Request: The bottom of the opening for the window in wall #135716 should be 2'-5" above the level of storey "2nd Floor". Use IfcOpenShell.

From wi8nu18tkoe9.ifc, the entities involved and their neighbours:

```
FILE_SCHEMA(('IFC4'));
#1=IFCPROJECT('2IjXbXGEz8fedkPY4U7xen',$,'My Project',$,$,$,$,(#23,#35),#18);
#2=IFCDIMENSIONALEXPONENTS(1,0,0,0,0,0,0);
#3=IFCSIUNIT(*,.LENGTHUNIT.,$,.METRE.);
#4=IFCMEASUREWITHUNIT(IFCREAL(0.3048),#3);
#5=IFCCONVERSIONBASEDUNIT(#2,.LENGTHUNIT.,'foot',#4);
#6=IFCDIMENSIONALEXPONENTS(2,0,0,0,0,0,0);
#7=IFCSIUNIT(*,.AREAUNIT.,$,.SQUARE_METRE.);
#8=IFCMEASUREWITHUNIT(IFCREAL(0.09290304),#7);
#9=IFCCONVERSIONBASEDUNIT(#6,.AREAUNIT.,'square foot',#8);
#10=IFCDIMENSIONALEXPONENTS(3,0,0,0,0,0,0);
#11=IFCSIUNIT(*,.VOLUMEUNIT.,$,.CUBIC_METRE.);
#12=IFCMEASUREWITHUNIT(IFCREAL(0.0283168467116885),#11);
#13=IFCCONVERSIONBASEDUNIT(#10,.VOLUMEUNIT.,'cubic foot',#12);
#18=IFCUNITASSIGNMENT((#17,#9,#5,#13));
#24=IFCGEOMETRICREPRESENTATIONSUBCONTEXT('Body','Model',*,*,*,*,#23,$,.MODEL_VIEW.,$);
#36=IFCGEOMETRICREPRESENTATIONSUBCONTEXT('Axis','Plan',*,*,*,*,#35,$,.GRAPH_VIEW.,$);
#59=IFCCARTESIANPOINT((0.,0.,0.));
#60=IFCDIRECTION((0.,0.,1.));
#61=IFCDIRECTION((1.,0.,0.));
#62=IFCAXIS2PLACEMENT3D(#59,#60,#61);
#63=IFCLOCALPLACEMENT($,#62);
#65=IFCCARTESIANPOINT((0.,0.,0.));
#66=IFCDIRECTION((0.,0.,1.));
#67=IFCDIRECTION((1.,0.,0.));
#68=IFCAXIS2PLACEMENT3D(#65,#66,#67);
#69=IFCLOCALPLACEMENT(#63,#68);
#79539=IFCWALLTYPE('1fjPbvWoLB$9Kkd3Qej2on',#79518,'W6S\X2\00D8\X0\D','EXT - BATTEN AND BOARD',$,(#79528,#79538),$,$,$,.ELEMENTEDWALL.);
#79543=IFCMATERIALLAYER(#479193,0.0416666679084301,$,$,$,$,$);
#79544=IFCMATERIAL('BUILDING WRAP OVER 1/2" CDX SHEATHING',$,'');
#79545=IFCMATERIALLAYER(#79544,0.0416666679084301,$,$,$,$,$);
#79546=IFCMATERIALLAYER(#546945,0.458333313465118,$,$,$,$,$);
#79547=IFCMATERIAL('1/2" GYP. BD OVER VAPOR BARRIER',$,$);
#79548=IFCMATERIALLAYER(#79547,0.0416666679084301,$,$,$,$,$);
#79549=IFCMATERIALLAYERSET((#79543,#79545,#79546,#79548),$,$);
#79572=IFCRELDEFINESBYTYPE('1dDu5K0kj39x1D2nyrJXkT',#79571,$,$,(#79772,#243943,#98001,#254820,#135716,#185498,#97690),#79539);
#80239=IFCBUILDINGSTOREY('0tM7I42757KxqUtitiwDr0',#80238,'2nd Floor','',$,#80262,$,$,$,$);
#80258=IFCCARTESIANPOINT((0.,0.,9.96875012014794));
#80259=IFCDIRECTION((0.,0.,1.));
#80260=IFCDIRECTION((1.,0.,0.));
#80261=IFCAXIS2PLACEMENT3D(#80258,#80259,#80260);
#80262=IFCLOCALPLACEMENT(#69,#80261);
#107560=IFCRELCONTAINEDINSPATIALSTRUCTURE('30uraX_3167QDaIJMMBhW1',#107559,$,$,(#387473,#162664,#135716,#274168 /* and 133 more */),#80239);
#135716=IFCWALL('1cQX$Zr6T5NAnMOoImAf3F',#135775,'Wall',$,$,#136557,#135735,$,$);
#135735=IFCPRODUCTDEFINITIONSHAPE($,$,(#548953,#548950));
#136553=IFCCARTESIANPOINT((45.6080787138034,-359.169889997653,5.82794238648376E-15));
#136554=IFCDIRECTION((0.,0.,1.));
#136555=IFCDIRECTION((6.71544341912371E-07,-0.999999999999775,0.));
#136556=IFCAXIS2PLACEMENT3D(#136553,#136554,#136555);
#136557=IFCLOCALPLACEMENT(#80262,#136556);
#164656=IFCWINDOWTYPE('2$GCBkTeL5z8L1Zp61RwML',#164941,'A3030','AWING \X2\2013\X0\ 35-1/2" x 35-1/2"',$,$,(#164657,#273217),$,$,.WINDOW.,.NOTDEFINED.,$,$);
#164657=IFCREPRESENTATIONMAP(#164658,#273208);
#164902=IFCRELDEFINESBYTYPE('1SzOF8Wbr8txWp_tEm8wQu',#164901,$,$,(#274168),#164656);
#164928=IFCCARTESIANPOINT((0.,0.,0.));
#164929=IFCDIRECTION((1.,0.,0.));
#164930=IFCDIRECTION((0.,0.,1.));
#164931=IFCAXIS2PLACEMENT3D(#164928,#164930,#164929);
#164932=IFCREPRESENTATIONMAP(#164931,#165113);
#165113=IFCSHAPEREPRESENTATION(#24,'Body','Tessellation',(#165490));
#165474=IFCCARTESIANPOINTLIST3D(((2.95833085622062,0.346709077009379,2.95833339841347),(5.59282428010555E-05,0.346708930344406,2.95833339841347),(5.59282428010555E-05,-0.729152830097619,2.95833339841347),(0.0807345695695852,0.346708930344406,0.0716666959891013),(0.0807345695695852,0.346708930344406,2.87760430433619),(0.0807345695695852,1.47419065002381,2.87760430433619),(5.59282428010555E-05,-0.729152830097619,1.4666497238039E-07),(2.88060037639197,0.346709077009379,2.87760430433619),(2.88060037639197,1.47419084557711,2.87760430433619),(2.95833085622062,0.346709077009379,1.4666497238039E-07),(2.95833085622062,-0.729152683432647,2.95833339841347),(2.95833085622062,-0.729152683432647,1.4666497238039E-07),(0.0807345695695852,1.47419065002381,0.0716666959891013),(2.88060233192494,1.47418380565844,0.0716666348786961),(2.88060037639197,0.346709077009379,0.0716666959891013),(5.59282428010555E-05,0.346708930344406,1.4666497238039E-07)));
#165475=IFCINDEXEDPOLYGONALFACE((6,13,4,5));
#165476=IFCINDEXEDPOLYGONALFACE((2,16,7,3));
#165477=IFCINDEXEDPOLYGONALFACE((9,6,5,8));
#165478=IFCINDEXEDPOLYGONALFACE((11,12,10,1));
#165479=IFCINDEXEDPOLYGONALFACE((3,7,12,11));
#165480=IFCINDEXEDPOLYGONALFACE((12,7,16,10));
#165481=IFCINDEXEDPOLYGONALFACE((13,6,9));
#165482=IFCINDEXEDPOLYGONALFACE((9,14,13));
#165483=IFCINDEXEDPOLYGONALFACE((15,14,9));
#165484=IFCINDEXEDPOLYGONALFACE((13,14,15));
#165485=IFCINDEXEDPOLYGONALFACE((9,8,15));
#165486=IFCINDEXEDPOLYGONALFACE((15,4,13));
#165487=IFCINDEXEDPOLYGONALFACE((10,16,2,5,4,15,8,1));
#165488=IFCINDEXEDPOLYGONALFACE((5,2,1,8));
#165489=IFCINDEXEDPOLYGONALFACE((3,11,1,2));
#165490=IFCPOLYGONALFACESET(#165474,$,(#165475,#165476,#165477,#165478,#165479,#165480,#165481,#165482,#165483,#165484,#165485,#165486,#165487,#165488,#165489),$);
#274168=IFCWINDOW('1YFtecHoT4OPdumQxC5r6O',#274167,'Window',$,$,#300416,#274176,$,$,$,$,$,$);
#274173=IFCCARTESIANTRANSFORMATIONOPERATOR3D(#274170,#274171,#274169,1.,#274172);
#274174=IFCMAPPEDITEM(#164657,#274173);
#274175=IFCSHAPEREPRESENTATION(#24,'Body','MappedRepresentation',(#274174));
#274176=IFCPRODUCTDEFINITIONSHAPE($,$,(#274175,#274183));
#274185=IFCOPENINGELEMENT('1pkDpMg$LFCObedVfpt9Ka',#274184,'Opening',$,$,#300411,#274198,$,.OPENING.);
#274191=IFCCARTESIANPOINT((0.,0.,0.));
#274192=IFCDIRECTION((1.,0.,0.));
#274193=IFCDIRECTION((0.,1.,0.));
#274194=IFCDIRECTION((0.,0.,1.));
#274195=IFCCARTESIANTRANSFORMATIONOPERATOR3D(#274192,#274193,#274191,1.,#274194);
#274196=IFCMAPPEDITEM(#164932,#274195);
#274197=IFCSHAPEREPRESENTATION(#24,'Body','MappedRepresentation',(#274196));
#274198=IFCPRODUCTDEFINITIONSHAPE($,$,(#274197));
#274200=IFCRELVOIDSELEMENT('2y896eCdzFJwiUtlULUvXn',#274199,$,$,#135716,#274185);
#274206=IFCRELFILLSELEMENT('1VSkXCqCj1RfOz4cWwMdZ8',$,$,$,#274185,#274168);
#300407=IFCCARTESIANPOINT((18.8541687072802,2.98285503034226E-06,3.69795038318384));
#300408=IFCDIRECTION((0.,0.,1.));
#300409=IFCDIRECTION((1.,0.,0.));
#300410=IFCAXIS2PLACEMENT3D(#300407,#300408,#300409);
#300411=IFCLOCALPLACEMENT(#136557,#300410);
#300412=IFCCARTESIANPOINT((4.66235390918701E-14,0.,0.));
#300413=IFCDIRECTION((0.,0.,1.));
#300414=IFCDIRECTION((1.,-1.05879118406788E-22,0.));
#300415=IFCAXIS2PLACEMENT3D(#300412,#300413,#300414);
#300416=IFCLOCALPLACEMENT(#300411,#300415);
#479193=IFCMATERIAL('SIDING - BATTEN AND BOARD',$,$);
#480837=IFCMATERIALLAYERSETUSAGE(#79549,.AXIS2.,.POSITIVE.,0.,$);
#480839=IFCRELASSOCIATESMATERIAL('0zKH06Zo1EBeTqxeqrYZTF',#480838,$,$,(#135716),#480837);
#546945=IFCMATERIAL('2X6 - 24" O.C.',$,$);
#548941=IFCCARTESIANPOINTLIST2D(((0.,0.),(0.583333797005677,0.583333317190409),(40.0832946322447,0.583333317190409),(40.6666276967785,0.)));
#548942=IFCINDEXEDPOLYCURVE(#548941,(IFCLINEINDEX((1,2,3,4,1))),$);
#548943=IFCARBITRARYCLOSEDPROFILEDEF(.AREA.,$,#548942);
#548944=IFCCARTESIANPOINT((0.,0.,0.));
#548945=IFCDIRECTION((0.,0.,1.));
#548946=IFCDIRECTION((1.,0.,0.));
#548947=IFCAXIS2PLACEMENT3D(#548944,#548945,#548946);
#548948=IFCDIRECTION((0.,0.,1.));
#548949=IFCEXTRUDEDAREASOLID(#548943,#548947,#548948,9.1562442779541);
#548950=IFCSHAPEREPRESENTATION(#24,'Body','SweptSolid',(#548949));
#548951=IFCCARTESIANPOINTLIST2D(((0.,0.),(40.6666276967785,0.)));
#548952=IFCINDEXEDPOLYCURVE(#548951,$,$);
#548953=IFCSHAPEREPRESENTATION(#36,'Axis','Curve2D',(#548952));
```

```python
import numpy as np
import ifcopenshell
import ifcopenshell.api.geometry
import ifcopenshell.geom
import ifcopenshell.util.element
import ifcopenshell.util.placement
import ifcopenshell.util.shape
import ifcopenshell.util.unit

model = ifcopenshell.open("wi8nu18tkoe9.ifc")
unit_scale = ifcopenshell.util.unit.calculate_unit_scale(model)

window = model.by_id(274168)
opening = window.FillsVoids[0].RelatingOpeningElement
storey = ifcopenshell.util.element.get_container(window, ifc_class="IfcBuildingStorey")
level = ifcopenshell.util.placement.get_local_placement(storey.ObjectPlacement)[2, 3]

# The opening's origin need not be at the sill, so measure its lowest point.
shape = ifcopenshell.geom.create_shape(ifcopenshell.geom.settings(), opening)
bottom = ifcopenshell.util.shape.get_shape_bottom_elevation(shape, shape.geometry) / unit_scale
dz = level + 29 * 0.0254 / unit_scale - bottom

shift = np.array([0.0, 0.0, dz])
# The window is placed relative to its opening, so it follows when the opening moves.
matrix = ifcopenshell.util.placement.get_local_placement(opening.ObjectPlacement)
matrix[:3, 3] += shift
ifcopenshell.api.geometry.edit_object_placement(
    model, product=opening, matrix=matrix, is_si=False, should_transform_children=True
)

print(f"moved by {dz * unit_scale:+.3f} m")

model.write("wi8nu18tkoe9_rev.ifc")
```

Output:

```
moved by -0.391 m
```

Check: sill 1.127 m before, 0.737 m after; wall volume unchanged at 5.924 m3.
